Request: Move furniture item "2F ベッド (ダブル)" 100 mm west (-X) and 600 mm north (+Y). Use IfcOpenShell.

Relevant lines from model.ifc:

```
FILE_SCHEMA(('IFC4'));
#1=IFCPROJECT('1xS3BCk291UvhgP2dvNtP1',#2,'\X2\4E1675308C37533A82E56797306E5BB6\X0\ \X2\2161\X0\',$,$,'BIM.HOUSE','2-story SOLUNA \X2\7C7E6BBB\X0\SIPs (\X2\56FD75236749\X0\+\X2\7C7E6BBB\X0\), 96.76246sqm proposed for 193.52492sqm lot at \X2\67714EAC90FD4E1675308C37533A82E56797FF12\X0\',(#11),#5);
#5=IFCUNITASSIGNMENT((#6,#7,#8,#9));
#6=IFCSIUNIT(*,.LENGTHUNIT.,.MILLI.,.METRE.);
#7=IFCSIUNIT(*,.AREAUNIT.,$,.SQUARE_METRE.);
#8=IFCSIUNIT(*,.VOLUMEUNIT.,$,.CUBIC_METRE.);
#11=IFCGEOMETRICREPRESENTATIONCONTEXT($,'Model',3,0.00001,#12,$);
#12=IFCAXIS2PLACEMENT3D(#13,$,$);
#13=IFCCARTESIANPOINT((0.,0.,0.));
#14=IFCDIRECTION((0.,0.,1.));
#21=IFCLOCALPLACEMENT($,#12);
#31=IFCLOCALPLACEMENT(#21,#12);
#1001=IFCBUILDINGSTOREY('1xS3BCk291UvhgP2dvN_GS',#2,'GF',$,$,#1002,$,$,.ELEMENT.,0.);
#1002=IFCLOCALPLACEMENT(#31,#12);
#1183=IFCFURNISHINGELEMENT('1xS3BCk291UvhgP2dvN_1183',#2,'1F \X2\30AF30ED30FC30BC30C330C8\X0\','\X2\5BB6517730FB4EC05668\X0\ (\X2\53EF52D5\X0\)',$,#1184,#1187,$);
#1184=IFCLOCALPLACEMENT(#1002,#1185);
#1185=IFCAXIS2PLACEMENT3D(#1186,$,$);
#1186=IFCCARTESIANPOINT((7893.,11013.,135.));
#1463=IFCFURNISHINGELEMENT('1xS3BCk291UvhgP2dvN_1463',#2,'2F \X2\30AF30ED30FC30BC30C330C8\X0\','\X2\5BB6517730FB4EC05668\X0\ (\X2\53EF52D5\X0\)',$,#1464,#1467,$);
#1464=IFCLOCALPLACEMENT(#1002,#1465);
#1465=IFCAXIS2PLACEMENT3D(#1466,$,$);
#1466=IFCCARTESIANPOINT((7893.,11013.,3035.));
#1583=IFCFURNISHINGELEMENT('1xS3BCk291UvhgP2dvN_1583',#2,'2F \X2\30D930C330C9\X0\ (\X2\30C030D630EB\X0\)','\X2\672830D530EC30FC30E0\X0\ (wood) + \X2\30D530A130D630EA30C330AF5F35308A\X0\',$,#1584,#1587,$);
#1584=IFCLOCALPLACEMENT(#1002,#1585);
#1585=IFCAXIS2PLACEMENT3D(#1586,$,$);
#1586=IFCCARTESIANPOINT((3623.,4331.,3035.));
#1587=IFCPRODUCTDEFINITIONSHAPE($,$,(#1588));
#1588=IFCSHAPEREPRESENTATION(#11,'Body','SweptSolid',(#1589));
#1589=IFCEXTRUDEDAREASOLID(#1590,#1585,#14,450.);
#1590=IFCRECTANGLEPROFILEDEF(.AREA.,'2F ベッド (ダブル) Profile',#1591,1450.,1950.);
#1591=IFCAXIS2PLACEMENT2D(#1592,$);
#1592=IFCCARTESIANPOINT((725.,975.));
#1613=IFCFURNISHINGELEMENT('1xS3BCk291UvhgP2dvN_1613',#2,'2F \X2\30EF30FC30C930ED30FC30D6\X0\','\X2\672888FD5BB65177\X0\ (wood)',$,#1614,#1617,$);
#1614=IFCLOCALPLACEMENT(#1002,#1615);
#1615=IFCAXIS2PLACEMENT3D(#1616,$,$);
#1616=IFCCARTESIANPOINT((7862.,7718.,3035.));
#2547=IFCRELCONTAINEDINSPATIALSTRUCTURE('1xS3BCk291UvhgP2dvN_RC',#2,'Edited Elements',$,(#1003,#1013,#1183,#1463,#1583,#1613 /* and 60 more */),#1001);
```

```python
import ifcopenshell
import ifcopenshell.api.geometry
import ifcopenshell.util.placement
import ifcopenshell.util.unit

model = ifcopenshell.open("model.ifc")
unit_scale = ifcopenshell.util.unit.calculate_unit_scale(model)

item = model.by_guid("1xS3BCk291UvhgP2dvN_1583")
matrix = ifcopenshell.util.placement.get_local_placement(item.ObjectPlacement)
matrix[0, 3] -= 0.1 / unit_scale
matrix[1, 3] += 0.6 / unit_scale
ifcopenshell.api.geometry.edit_object_placement(model, product=item, matrix=matrix, is_si=False)

print(ifcopenshell.util.placement.get_local_placement(item.ObjectPlacement).round(3) + 0.0)

model.write("model_updated.ifc")
```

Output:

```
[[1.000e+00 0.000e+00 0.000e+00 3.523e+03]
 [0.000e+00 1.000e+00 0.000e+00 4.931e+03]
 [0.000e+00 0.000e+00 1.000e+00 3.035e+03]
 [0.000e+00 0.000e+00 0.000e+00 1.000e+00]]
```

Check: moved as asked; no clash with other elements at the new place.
